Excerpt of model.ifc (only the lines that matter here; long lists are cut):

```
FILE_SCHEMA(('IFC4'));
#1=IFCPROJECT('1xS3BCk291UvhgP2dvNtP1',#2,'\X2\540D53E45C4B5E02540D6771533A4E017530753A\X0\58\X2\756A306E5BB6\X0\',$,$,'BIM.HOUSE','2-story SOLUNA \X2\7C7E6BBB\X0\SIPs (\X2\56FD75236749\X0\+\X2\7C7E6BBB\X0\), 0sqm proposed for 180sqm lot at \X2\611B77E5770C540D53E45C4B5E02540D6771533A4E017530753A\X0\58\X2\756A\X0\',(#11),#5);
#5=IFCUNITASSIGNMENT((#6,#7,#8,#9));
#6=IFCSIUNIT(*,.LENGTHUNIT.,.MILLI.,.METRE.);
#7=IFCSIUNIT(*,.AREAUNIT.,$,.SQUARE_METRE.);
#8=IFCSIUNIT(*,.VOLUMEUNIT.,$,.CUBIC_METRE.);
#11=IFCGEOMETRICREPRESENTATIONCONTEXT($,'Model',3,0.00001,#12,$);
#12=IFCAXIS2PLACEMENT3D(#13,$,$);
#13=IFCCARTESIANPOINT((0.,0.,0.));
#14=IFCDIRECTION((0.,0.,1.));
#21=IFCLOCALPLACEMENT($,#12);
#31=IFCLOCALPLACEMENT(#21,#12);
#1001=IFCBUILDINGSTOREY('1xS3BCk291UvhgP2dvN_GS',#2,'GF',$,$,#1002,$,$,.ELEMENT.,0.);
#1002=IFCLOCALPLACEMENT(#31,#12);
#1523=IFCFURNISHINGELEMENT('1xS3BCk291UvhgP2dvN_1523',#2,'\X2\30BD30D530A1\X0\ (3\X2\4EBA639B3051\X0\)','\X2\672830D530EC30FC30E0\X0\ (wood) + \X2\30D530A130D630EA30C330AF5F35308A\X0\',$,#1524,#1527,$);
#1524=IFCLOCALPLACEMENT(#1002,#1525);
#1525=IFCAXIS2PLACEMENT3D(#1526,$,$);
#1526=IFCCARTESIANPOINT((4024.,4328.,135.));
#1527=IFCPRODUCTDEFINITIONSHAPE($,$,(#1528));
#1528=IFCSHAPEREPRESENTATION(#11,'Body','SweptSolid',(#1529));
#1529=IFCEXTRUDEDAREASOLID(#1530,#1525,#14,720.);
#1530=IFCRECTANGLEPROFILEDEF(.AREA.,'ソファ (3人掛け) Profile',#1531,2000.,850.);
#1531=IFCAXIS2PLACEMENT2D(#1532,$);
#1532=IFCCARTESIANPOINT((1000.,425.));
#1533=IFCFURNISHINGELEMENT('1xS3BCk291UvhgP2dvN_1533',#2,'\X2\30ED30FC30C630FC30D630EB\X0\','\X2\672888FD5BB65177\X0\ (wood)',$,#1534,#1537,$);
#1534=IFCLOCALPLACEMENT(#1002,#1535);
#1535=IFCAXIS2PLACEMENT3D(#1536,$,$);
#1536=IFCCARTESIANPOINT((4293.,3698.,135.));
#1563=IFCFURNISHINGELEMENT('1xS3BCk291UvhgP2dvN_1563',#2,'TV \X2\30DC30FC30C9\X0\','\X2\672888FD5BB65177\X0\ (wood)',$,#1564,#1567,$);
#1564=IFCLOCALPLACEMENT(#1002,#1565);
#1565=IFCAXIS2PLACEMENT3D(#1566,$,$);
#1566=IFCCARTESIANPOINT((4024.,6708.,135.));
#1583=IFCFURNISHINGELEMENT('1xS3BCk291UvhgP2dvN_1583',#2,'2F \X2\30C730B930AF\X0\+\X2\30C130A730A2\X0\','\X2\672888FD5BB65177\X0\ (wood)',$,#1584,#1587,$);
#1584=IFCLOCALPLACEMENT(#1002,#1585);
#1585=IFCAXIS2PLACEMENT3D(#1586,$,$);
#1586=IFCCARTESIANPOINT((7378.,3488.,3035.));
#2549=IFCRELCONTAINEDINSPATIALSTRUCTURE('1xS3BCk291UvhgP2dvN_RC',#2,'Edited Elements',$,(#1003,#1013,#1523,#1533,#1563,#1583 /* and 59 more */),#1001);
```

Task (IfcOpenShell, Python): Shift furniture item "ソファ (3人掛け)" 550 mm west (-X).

```python
import ifcopenshell
import ifcopenshell.api.geometry
import ifcopenshell.util.placement

model = ifcopenshell.open("model.ifc")

item = model.by_guid("1xS3BCk291UvhgP2dvN_1523")
matrix = ifcopenshell.util.placement.get_local_placement(item.ObjectPlacement)
matrix[0, 3] -= 550.0
ifcopenshell.api.geometry.edit_object_placement(model, product=item, matrix=matrix, is_si=False)

print(ifcopenshell.util.placement.get_local_placement(item.ObjectPlacement).round(3) + 0.0)

model.write("model_updated.ifc")
```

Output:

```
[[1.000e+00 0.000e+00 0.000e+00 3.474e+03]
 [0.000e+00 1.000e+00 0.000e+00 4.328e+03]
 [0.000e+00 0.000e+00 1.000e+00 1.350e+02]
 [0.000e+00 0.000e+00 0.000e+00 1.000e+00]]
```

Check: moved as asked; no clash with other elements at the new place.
